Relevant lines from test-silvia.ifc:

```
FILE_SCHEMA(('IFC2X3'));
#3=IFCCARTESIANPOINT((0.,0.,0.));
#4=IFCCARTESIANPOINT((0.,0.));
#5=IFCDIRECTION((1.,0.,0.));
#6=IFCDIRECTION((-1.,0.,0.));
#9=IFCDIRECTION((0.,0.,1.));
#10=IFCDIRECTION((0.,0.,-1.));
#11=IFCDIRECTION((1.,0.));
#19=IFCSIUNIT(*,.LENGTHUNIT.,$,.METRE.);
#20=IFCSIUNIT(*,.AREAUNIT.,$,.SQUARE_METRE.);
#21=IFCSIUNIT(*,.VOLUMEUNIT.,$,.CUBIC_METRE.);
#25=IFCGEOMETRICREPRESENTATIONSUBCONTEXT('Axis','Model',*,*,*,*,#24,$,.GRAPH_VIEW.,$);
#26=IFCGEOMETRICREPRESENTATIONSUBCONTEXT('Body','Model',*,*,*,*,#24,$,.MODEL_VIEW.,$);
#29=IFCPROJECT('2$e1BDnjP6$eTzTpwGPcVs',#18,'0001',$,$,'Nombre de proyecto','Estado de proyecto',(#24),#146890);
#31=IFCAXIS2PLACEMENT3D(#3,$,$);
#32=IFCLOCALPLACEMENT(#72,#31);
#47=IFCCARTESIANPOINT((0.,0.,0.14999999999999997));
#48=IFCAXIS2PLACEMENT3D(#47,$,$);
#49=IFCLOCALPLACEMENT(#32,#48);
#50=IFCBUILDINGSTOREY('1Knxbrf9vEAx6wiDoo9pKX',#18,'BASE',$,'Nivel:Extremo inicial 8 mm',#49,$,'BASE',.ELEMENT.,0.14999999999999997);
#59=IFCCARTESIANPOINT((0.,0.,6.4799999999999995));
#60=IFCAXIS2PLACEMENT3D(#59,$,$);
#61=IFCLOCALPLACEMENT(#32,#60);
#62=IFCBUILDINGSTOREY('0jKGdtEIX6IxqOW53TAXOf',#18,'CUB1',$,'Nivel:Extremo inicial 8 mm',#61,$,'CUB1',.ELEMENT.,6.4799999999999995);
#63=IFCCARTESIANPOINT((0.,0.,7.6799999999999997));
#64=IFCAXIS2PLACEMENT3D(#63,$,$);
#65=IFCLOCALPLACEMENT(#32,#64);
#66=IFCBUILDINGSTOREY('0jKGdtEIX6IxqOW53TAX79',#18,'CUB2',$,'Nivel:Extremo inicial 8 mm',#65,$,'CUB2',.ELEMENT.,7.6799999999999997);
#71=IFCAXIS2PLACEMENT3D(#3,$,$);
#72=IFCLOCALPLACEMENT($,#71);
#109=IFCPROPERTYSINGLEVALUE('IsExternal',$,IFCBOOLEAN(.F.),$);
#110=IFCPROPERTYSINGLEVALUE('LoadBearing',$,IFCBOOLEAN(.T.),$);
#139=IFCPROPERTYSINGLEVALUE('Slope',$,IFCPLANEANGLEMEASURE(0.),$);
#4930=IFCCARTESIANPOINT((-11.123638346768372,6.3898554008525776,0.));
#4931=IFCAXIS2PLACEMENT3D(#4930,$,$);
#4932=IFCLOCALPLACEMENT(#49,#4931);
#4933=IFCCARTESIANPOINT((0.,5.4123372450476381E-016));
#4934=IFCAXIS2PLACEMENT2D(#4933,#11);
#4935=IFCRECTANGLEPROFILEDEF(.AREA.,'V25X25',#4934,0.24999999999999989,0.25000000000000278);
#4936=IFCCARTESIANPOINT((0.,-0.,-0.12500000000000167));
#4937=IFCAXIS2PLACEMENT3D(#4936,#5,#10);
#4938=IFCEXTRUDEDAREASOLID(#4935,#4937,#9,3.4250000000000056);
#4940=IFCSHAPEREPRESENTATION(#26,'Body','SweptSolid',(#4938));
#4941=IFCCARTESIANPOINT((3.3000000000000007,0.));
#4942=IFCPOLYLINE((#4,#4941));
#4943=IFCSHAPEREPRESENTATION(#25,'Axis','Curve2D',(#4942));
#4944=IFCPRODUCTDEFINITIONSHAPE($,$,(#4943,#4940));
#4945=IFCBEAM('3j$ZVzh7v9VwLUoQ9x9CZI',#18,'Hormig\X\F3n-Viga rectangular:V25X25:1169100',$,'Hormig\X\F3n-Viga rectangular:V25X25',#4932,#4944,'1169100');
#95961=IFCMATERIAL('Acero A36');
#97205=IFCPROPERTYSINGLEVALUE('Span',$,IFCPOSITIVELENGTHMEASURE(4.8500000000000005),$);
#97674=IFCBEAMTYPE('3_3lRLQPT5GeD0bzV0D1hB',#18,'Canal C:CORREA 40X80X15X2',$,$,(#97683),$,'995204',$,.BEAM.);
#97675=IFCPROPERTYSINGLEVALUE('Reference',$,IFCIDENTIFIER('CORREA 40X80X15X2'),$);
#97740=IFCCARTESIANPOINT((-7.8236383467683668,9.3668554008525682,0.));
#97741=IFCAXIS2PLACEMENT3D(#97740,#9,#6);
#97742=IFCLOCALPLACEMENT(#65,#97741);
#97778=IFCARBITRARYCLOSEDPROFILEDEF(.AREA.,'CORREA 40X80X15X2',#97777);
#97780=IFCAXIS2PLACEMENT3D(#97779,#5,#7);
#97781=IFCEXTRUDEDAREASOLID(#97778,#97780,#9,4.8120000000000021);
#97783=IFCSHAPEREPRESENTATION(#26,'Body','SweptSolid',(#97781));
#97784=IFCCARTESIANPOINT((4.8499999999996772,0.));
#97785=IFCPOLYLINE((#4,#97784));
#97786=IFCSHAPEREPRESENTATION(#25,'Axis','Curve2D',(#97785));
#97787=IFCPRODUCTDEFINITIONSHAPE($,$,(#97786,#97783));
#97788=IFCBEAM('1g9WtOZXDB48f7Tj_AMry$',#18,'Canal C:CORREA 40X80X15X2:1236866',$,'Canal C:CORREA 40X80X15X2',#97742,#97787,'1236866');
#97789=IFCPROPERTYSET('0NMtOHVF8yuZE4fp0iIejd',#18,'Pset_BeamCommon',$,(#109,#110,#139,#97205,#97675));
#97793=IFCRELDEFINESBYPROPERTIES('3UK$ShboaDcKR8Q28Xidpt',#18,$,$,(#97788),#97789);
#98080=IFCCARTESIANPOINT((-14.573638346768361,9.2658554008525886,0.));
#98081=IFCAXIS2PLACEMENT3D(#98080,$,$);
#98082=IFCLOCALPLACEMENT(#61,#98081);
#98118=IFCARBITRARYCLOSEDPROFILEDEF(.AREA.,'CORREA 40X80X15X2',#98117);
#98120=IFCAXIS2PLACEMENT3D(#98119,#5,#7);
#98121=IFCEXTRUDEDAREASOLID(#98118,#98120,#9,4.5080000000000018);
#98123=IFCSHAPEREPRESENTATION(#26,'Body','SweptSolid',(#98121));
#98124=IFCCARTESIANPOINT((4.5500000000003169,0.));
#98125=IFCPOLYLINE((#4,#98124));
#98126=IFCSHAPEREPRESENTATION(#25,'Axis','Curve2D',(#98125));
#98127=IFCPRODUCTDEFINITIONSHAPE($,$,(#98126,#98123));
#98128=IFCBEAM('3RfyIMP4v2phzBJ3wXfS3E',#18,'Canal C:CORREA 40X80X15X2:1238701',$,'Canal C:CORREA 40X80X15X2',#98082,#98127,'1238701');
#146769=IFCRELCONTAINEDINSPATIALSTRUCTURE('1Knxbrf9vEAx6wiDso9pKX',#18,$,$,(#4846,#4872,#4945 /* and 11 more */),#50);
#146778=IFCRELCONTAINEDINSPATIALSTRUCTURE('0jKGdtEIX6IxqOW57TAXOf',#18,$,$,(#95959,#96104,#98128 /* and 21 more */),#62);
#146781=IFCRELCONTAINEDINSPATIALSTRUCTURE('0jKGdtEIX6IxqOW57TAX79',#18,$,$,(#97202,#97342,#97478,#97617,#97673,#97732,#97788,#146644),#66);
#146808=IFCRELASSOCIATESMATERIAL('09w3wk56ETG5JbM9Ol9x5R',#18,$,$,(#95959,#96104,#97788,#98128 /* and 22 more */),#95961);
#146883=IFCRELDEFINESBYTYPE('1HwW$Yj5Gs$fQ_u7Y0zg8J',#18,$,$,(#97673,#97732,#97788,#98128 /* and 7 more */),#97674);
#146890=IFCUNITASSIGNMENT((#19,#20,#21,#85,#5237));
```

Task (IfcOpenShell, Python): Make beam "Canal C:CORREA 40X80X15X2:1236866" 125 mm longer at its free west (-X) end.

```python
import numpy as np
import ifcopenshell
import ifcopenshell.api.pset
import ifcopenshell.util.element
import ifcopenshell.util.representation

model = ifcopenshell.open("test-silvia.ifc")

member = model.by_guid("1g9WtOZXDB48f7Tj_AMry$")
change = 0.125

# The extrusion runs towards the end named, so only its depth changes.
body = ifcopenshell.util.representation.get_representation(member, "Model", "Body")
solid = body.Items[0]
old_length = solid.Depth
solid.Depth += change

# Move the axis end point with it.
axis = next(r for r in member.Representation.Representations if r.RepresentationIdentifier == "Axis").Items[0]
start, end = (np.array(p.Coordinates) for p in axis.Points)
end = end + (end - start) / np.linalg.norm(end - start) * change
point = model.createIfcCartesianPoint(end.tolist())
axis.Points = [axis.Points[0], point]

# Update the stored length and volume.
pset = model.by_id(ifcopenshell.util.element.get_pset(member, "Pset_BeamCommon", should_inherit=False)["id"])
ifcopenshell.api.pset.edit_pset(model, pset=pset, properties={
    "Span": model.create_entity("IfcPositiveLengthMeasure", solid.Depth),
})

print(f"length {old_length:g} -> {solid.Depth:g}")

model.write("test-silvia_v2.ifc")
```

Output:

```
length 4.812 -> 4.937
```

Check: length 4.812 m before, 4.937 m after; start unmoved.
